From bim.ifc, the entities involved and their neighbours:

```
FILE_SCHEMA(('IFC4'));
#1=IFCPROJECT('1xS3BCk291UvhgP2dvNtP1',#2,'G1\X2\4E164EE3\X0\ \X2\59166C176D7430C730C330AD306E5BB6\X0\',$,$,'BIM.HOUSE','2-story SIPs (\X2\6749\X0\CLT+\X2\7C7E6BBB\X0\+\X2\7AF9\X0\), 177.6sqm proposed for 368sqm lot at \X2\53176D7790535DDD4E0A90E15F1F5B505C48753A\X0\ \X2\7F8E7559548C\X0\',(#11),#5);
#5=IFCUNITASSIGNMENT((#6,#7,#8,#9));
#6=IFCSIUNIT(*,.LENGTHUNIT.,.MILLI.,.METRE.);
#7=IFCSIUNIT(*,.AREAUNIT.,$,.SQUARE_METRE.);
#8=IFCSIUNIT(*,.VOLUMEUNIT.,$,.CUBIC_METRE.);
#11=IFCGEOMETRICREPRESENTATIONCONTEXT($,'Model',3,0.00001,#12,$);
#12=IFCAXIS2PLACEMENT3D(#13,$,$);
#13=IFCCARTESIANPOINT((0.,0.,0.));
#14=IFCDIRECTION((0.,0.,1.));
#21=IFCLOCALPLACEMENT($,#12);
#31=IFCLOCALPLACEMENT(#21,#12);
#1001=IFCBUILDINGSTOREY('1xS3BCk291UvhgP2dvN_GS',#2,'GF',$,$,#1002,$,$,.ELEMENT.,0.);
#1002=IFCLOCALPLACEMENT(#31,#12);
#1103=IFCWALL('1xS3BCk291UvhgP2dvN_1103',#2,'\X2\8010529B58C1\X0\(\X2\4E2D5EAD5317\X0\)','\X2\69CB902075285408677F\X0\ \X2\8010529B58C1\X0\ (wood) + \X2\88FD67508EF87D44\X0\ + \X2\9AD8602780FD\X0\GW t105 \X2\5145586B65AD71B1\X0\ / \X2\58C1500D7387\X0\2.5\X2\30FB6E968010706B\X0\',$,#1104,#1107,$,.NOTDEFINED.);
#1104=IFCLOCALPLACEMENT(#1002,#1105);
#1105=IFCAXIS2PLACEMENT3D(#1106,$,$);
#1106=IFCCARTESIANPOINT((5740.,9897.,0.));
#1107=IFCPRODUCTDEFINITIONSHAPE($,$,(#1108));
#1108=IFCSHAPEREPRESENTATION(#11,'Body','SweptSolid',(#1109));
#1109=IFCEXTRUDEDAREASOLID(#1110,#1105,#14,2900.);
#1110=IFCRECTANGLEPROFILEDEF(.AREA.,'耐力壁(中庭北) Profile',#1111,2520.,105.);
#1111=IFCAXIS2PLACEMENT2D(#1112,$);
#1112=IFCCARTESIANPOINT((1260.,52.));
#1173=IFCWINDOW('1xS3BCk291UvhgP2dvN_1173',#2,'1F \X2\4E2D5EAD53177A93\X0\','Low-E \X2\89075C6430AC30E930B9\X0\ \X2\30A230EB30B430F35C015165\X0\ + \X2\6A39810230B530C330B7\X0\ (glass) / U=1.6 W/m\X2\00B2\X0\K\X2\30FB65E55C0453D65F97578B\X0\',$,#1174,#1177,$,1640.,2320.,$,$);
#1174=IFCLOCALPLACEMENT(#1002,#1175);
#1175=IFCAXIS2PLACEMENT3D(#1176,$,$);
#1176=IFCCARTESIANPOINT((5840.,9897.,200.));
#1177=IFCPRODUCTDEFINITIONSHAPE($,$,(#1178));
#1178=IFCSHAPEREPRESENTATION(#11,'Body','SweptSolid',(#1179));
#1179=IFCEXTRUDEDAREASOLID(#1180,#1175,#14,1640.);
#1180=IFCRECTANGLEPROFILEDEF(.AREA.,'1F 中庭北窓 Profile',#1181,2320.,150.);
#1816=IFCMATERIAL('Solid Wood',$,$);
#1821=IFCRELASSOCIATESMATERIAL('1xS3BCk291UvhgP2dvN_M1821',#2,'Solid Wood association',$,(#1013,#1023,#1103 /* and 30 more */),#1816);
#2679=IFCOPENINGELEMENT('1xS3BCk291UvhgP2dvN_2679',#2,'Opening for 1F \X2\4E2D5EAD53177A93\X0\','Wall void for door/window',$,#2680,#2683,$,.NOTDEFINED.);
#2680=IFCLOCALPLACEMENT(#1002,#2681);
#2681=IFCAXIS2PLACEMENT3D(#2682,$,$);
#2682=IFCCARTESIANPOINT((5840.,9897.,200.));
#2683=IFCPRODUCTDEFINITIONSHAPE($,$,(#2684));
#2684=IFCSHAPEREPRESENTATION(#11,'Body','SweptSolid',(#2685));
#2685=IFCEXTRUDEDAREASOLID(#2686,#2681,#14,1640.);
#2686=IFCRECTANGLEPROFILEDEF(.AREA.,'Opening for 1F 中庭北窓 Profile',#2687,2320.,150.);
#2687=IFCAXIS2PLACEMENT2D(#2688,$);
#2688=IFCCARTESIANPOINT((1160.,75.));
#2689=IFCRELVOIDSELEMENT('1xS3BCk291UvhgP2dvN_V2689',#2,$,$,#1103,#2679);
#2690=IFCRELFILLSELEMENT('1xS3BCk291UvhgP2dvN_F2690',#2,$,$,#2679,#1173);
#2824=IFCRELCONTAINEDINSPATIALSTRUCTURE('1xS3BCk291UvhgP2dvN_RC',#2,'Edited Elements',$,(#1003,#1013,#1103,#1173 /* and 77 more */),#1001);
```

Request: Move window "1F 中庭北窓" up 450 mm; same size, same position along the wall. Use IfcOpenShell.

```python
import numpy as np
import ifcopenshell
import ifcopenshell.api.geometry
import ifcopenshell.util.placement
import ifcopenshell.util.unit

model = ifcopenshell.open("bim.ifc")
unit_scale = ifcopenshell.util.unit.calculate_unit_scale(model)

window = model.by_guid("1xS3BCk291UvhgP2dvN_1173")
opening = window.FillsVoids[0].RelatingOpeningElement
dz = 450.0

shift = np.array([0.0, 0.0, dz])
# The window is not placed relative to its opening, so move both.
for product in (opening, window):
    matrix = ifcopenshell.util.placement.get_local_placement(product.ObjectPlacement)
    matrix[:3, 3] += shift
    ifcopenshell.api.geometry.edit_object_placement(model, product=product, matrix=matrix, is_si=False)

print(f"moved by {dz * unit_scale:+.3f} m")

model.write("bim_v2.ifc")
```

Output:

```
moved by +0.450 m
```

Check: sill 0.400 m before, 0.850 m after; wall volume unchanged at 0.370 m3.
